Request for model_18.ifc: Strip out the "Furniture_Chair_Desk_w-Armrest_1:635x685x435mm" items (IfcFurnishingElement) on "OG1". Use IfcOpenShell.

First a look at what the model holds.

```python
import ifcopenshell
import ifcopenshell.util.element

model = ifcopenshell.open("model_18.ifc")
print(model.schema)
storey = next(s for s in model.by_type("IfcBuildingStorey") if s.Name == "OG1")
furniture = [e for e in ifcopenshell.util.element.get_decomposition(storey) if e.is_a("IfcFurnishingElement")]
seen = {}
for e in furniture:
    element_type = ifcopenshell.util.element.get_type(e)
    name = element_type.Name if element_type not in (None, e) else None
    seen[name] = seen.get(name, 0) + 1
for name, count in sorted(seen.items(), key=str):
    print(count, "x", name)
```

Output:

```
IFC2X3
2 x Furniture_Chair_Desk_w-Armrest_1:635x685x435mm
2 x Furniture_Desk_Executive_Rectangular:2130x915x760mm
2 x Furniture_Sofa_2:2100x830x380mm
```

```python
import ifcopenshell
import ifcopenshell.api.root
import ifcopenshell.util.element

model = ifcopenshell.open("model_18.ifc")

storey = next(s for s in model.by_type("IfcBuildingStorey") if s.Name == "OG1")
furniture = [e for e in ifcopenshell.util.element.get_decomposition(storey) if e.is_a("IfcFurnishingElement")]
targets = [e for e in furniture if (t := ifcopenshell.util.element.get_type(e)) not in (None, e) and t.Name == "Furniture_Chair_Desk_w-Armrest_1:635x685x435mm"]

for e in targets:
    ifcopenshell.api.root.remove_product(model, product=e)
print(len(targets), "removed")

model.write("model_18_v2.ifc")
```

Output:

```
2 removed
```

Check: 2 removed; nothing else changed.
